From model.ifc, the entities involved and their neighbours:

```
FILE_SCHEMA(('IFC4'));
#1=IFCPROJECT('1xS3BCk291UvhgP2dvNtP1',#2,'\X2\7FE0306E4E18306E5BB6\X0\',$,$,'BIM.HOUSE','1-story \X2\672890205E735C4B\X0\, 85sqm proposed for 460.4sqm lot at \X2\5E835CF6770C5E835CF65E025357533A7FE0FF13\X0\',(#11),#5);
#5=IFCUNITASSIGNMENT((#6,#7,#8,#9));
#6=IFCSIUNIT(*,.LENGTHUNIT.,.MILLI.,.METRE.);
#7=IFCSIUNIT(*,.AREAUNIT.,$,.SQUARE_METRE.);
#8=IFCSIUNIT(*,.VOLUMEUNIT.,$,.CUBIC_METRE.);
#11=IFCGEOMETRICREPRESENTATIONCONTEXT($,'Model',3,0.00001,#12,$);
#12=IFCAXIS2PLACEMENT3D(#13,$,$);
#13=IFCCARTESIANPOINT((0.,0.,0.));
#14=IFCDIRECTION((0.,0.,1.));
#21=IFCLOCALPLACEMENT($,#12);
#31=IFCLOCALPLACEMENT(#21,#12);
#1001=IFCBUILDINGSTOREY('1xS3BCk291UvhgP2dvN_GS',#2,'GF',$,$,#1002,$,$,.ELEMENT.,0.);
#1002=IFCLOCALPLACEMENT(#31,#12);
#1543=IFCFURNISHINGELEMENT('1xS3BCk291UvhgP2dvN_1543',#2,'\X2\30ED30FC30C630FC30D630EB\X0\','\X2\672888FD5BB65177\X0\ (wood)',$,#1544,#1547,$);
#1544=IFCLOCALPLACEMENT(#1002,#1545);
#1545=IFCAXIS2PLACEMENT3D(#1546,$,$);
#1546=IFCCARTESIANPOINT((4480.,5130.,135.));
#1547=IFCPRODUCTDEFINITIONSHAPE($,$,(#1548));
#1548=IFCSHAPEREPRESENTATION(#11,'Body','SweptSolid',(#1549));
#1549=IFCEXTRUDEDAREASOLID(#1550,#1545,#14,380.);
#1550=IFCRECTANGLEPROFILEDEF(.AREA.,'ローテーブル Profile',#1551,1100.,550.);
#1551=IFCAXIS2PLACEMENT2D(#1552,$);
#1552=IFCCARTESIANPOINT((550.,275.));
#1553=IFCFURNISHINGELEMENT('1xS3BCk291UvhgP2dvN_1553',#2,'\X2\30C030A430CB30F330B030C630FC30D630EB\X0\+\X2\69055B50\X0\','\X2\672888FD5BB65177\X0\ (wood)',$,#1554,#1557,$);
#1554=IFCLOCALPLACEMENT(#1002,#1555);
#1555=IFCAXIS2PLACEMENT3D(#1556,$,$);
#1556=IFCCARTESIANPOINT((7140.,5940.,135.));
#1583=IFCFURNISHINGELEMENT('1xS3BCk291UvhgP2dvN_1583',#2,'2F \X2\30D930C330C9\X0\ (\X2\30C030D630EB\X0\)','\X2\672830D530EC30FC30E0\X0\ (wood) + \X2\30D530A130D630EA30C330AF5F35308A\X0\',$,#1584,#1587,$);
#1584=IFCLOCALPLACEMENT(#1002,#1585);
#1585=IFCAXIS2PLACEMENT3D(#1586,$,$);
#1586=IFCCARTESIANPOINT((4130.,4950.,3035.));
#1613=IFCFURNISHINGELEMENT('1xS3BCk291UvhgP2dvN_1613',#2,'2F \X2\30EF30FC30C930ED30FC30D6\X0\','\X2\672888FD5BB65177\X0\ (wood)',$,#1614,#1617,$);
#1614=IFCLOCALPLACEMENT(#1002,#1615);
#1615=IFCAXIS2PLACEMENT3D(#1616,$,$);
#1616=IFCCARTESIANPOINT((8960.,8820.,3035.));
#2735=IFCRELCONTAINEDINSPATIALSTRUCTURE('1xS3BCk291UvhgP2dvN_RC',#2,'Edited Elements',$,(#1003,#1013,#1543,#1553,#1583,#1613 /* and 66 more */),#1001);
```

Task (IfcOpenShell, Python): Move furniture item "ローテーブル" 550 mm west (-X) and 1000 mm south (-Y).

```python
import ifcopenshell
import ifcopenshell.api.geometry
import ifcopenshell.util.placement
import ifcopenshell.util.unit

model = ifcopenshell.open("model.ifc")
unit_scale = ifcopenshell.util.unit.calculate_unit_scale(model)

item = model.by_guid("1xS3BCk291UvhgP2dvN_1543")
matrix = ifcopenshell.util.placement.get_local_placement(item.ObjectPlacement)
matrix[0, 3] -= 0.55 / unit_scale
matrix[1, 3] -= 1 / unit_scale
ifcopenshell.api.geometry.edit_object_placement(model, product=item, matrix=matrix, is_si=False)

print(ifcopenshell.util.placement.get_local_placement(item.ObjectPlacement).round(3) + 0.0)

model.write("model_v2.ifc")
```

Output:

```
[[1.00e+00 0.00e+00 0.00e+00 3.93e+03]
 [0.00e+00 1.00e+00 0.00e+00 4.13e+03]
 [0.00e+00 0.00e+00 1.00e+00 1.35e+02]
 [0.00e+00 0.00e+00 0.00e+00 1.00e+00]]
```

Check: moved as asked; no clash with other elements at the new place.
